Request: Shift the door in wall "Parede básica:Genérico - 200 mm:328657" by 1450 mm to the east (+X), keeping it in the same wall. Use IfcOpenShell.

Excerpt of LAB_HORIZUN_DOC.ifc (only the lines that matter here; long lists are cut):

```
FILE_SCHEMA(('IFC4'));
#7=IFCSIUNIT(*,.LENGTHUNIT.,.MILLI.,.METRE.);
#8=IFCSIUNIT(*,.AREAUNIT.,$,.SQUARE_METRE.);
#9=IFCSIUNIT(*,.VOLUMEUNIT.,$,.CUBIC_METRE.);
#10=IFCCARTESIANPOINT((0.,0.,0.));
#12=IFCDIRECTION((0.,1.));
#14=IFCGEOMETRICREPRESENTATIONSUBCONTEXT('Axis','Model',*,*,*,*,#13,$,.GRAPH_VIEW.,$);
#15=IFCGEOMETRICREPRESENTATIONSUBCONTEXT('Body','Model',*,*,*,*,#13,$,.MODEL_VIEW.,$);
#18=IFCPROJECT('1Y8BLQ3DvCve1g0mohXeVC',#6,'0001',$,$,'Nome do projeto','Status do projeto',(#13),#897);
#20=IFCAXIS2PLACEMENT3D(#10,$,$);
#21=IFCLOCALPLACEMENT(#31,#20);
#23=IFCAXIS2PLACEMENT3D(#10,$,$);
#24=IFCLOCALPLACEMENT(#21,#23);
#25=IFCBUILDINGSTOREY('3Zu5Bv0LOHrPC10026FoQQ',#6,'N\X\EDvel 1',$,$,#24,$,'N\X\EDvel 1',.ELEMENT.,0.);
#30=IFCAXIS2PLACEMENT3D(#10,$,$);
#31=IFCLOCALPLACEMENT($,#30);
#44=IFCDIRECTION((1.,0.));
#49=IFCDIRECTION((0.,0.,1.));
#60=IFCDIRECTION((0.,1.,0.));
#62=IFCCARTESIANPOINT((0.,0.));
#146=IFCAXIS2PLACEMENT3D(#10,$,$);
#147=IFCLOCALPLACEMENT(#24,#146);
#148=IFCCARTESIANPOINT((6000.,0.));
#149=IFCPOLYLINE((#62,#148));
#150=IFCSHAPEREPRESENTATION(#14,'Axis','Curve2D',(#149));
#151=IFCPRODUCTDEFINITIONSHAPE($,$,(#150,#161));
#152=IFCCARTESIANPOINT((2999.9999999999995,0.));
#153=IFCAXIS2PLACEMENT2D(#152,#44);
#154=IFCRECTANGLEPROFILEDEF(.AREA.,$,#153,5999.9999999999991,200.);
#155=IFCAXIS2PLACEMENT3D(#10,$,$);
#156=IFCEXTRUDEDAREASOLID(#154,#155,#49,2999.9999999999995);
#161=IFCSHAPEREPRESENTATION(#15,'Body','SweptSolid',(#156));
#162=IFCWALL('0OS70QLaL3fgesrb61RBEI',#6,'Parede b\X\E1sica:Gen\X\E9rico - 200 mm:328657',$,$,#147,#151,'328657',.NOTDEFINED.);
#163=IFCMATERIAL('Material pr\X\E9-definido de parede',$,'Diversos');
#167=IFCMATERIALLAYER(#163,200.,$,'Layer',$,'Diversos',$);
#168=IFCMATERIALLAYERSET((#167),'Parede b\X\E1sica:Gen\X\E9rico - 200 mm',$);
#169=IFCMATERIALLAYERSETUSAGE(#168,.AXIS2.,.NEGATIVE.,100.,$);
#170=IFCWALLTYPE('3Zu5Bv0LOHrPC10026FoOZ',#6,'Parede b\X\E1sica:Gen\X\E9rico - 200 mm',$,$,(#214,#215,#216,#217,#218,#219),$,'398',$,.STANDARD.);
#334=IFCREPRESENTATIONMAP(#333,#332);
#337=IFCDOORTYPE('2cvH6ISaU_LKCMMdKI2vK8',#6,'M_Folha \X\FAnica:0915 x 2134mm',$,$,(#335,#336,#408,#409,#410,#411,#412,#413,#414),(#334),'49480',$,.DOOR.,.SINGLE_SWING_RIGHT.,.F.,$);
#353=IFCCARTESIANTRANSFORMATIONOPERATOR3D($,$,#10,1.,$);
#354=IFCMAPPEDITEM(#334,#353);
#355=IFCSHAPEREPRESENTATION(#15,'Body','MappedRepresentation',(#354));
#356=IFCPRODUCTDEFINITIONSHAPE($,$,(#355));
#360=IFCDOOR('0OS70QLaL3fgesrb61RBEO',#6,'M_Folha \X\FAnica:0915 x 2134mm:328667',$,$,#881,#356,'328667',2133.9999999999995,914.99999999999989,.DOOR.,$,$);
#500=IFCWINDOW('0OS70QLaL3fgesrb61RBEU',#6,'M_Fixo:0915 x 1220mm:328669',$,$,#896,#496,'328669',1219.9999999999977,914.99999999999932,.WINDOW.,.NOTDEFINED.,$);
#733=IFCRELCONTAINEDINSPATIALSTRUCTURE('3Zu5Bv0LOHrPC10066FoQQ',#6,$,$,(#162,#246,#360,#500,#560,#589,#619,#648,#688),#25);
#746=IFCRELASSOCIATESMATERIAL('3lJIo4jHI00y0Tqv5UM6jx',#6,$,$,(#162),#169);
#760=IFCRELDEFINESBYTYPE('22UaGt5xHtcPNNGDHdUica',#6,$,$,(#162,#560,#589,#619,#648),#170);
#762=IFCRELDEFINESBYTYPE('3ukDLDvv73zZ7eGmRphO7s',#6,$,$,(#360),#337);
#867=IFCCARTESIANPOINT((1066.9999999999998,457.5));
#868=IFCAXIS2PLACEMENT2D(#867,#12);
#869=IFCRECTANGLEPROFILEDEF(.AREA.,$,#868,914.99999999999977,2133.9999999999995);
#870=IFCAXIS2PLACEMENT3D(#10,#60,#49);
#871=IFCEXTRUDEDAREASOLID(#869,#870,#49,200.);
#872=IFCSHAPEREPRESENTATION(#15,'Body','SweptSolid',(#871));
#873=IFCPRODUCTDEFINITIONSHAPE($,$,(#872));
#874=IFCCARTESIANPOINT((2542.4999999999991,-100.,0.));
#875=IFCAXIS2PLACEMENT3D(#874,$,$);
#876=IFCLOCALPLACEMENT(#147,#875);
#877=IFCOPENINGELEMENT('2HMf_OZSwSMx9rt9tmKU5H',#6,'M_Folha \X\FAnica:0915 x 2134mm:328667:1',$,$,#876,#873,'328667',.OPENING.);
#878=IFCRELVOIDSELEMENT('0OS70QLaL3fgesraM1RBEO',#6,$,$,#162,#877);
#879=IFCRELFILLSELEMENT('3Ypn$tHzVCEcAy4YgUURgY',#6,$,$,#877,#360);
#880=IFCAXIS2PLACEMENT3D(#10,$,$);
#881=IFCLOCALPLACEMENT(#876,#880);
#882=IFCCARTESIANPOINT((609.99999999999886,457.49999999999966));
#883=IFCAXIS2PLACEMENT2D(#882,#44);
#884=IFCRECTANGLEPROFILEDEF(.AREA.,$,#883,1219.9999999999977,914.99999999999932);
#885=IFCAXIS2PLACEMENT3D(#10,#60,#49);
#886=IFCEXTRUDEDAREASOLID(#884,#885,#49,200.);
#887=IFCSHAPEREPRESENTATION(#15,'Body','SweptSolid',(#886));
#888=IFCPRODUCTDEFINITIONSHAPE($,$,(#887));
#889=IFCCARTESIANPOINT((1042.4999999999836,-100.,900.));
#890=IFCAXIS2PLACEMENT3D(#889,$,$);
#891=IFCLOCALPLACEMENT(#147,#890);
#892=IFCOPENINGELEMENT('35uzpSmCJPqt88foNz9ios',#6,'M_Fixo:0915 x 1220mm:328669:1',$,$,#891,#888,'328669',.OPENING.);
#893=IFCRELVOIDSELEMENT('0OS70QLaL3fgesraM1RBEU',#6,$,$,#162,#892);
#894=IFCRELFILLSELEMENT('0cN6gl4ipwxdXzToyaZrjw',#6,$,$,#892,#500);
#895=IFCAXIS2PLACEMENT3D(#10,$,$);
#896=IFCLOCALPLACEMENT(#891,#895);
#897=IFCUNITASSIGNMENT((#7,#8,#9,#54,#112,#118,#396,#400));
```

```python
import ifcopenshell
import ifcopenshell.api.geometry
import ifcopenshell.util.placement
import ifcopenshell.util.unit

model = ifcopenshell.open("LAB_HORIZUN_DOC.ifc")
unit_scale = ifcopenshell.util.unit.calculate_unit_scale(model)

door = model.by_guid("0OS70QLaL3fgesrb61RBEO")
opening = door.FillsVoids[0].RelatingOpeningElement
wall = opening.VoidsElements[0].RelatingBuildingElement

wall_matrix = ifcopenshell.util.placement.get_local_placement(wall.ObjectPlacement)
shift = wall_matrix[:3, 0] * 1.45 / unit_scale
before = ifcopenshell.util.placement.get_local_placement(door.ObjectPlacement)[:3, 3].copy()

# The door is placed relative to its opening, so it follows when the opening moves.
matrix = ifcopenshell.util.placement.get_local_placement(opening.ObjectPlacement)
matrix[:3, 3] += shift
ifcopenshell.api.geometry.edit_object_placement(
    model, product=opening, matrix=matrix, is_si=False, should_transform_children=True
)

after = ifcopenshell.util.placement.get_local_placement(door.ObjectPlacement)[:3, 3]
print("door moved by", (after - before).round(3) + 0.0)

model.write("LAB_HORIZUN_DOC_edited.ifc")
```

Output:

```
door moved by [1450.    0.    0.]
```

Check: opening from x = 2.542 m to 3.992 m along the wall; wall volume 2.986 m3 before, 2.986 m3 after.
